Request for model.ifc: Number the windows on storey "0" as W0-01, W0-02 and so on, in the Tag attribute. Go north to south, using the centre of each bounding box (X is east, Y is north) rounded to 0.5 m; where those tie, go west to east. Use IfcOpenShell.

First a look at what the model holds.

```python
import ifcopenshell
import ifcopenshell.util.element
import ifcopenshell.util.placement

model = ifcopenshell.open("model.ifc")
print(model.schema)
storey = next(s for s in model.by_type("IfcBuildingStorey") if s.Name == "0")
windows = [e for e in ifcopenshell.util.element.get_decomposition(storey) if e.is_a("IfcWindow")]
for e in sorted(windows, key=lambda e: e.id()):
    origin = ifcopenshell.util.placement.get_local_placement(e.ObjectPlacement)[:3, 3]
    print(e.id(), e.Tag, e.Name, origin.round(2) + 0.0, sep=" | ")
```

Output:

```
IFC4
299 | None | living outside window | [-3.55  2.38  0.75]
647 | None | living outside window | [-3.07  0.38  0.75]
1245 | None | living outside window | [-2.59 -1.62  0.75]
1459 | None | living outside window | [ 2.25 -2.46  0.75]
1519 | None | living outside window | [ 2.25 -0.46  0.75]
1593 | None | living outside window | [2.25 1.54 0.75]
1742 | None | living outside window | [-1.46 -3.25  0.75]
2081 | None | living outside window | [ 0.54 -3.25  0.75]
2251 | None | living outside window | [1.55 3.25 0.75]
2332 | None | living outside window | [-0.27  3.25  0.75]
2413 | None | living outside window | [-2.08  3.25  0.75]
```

```python
import ifcopenshell
import ifcopenshell.geom
import ifcopenshell.util.element
import ifcopenshell.util.shape

model = ifcopenshell.open("model.ifc")
settings = ifcopenshell.geom.settings()
settings.set("use-world-coords", True)


def centre(element):
    shape = ifcopenshell.geom.create_shape(settings, element)
    return ifcopenshell.util.shape.get_bbox_centroid(shape.geometry)


storey = next(s for s in model.by_type("IfcBuildingStorey") if s.Name == "0")
windows = [e for e in ifcopenshell.util.element.get_decomposition(storey) if e.is_a("IfcWindow")]

# Insertion points can sit at a corner or the storey origin, so sort by the geometry (in metres).
centres = {e: centre(e) for e in windows}
windows.sort(key=lambda e: (-round(centres[e][1] / 0.5), centres[e][0]))

for i, e in enumerate(windows, start=1):
    number = f"W0-{i:02d}"
    e.Tag = number
    print(e.id(), number)

model.write("model_edited.ifc")
```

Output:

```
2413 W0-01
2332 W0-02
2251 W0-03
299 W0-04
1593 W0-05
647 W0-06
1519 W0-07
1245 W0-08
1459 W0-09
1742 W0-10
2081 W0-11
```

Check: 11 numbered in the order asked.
